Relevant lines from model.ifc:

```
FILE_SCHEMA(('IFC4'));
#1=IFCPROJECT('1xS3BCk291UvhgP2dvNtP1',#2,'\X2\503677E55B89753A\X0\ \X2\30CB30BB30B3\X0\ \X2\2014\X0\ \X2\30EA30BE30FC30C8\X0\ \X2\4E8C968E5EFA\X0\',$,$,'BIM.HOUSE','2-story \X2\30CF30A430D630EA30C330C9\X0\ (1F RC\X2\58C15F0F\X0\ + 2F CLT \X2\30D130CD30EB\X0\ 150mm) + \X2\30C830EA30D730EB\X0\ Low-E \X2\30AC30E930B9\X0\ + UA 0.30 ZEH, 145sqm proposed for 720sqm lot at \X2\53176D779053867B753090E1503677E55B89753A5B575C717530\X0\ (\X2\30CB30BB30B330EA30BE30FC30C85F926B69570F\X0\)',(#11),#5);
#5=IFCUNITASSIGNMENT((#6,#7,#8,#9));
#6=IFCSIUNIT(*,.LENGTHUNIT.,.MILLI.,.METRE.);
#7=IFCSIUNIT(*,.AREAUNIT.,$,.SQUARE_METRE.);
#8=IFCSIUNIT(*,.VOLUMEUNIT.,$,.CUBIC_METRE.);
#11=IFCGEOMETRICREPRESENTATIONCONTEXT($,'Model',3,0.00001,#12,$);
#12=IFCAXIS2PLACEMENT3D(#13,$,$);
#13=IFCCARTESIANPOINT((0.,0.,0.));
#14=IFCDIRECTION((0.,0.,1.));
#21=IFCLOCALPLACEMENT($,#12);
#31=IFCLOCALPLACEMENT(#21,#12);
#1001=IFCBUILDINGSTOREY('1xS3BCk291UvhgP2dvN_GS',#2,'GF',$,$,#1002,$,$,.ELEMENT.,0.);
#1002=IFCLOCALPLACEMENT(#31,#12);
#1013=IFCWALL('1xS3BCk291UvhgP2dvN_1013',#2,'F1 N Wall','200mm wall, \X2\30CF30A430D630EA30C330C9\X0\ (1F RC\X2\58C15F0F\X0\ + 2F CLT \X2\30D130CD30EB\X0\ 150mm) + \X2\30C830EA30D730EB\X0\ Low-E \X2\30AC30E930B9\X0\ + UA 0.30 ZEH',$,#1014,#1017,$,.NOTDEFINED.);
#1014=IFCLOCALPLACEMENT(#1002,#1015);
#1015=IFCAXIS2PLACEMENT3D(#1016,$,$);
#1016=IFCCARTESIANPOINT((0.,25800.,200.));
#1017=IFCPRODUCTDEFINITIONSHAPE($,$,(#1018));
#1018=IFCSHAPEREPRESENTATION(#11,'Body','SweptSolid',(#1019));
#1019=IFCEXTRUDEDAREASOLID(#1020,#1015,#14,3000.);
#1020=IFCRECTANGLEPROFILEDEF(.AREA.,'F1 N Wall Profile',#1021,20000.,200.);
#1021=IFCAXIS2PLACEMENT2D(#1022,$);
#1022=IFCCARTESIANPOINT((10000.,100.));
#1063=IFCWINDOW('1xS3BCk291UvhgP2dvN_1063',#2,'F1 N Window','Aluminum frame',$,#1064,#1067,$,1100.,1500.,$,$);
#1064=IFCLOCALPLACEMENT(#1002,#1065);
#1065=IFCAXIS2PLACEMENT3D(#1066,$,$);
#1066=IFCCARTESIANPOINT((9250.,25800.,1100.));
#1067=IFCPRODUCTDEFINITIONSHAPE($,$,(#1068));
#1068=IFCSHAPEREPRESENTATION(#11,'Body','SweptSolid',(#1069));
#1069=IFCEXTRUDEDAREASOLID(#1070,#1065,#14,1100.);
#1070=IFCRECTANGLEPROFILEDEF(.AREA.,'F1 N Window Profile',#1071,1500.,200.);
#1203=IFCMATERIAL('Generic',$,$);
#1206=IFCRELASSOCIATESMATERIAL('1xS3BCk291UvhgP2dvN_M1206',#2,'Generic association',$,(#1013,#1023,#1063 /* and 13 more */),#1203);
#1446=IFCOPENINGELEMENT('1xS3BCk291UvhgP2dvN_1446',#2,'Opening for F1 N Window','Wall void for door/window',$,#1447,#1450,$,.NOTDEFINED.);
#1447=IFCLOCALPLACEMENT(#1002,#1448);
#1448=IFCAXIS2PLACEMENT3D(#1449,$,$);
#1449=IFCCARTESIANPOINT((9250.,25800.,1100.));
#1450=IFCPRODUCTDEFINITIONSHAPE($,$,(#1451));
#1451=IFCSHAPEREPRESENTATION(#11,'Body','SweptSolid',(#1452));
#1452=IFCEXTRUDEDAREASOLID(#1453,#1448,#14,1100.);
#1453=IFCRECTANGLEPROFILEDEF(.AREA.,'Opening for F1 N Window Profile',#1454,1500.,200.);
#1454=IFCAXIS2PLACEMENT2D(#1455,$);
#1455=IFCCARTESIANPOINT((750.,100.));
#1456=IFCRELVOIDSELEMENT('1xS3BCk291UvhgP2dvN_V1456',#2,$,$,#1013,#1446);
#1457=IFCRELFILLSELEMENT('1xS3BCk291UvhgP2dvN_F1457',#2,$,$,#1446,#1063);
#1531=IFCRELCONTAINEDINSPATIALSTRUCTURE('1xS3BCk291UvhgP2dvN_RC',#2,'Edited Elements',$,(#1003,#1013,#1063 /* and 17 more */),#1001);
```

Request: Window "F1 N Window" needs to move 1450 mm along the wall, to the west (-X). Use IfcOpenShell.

```python
import ifcopenshell
import ifcopenshell.api.geometry
import ifcopenshell.util.placement
import ifcopenshell.util.unit

model = ifcopenshell.open("model.ifc")
unit_scale = ifcopenshell.util.unit.calculate_unit_scale(model)

window = model.by_guid("1xS3BCk291UvhgP2dvN_1063")
opening = window.FillsVoids[0].RelatingOpeningElement
wall = opening.VoidsElements[0].RelatingBuildingElement

wall_matrix = ifcopenshell.util.placement.get_local_placement(wall.ObjectPlacement)
shift = wall_matrix[:3, 0] * -1.45 / unit_scale
before = ifcopenshell.util.placement.get_local_placement(window.ObjectPlacement)[:3, 3].copy()

# The window is not placed relative to its opening, so move both.
for product in (opening, window):
    matrix = ifcopenshell.util.placement.get_local_placement(product.ObjectPlacement)
    matrix[:3, 3] += shift
    ifcopenshell.api.geometry.edit_object_placement(model, product=product, matrix=matrix, is_si=False)

after = ifcopenshell.util.placement.get_local_placement(window.ObjectPlacement)[:3, 3]
print("window moved by", (after - before).round(3) + 0.0)

model.write("model_updated.ifc")
```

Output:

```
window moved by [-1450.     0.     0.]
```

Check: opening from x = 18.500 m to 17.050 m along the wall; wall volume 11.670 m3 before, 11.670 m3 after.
